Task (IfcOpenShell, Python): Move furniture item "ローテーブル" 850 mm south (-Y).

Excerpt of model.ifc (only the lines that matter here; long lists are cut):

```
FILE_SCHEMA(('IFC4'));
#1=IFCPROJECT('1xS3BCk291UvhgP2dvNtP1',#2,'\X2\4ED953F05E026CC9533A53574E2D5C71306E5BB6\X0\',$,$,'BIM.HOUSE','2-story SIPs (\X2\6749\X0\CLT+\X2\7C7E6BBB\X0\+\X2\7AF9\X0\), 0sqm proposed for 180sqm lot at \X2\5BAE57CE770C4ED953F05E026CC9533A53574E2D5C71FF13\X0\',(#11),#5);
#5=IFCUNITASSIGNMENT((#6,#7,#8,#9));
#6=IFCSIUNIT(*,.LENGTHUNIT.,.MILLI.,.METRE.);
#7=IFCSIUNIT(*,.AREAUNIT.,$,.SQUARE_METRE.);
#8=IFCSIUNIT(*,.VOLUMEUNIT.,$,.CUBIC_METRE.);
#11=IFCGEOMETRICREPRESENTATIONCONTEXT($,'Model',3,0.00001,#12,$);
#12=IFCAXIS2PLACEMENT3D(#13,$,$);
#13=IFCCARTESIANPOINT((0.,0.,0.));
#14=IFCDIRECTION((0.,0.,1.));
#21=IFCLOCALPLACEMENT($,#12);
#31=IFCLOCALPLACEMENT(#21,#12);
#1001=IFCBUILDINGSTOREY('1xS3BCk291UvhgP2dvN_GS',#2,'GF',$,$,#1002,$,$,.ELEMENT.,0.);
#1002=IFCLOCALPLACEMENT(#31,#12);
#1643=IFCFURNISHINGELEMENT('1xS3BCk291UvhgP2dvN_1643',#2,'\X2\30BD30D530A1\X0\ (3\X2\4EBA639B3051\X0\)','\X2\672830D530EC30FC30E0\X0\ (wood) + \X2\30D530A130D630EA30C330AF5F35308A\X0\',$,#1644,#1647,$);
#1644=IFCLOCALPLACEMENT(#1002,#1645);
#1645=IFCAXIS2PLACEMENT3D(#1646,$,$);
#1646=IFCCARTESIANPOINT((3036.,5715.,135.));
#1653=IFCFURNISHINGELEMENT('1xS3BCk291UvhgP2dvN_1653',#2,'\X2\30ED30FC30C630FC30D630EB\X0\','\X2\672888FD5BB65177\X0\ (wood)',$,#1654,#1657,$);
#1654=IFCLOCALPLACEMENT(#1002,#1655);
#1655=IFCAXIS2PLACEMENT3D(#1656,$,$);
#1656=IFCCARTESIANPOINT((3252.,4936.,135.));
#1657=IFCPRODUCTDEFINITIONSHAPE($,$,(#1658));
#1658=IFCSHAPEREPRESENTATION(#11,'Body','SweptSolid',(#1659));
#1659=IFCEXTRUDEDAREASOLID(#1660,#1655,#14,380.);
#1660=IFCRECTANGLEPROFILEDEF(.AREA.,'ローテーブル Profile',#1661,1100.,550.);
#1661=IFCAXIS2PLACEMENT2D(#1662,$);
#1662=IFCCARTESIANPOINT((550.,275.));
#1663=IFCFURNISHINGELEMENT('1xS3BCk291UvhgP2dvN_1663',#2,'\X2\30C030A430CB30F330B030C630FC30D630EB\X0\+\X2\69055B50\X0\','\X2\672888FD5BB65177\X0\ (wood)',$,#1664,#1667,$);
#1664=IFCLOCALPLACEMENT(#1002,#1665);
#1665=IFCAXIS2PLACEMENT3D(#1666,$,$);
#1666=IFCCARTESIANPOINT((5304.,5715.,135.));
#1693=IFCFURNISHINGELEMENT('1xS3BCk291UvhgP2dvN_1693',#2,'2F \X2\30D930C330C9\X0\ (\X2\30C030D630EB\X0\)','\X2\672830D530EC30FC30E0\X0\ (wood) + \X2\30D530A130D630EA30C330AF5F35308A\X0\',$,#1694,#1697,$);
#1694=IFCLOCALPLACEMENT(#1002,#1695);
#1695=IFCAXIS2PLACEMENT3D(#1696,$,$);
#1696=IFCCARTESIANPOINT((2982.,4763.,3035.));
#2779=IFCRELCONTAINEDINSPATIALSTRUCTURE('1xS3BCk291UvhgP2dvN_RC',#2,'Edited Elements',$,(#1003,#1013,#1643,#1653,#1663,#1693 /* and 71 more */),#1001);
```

```python
import ifcopenshell
import ifcopenshell.api.geometry
import ifcopenshell.util.placement
import ifcopenshell.util.unit

model = ifcopenshell.open("model.ifc")
unit_scale = ifcopenshell.util.unit.calculate_unit_scale(model)

item = model.by_guid("1xS3BCk291UvhgP2dvN_1653")
matrix = ifcopenshell.util.placement.get_local_placement(item.ObjectPlacement)
matrix[1, 3] -= 0.85 / unit_scale
ifcopenshell.api.geometry.edit_object_placement(model, product=item, matrix=matrix, is_si=False)

print(ifcopenshell.util.placement.get_local_placement(item.ObjectPlacement).round(3) + 0.0)

model.write("model_rev.ifc")
```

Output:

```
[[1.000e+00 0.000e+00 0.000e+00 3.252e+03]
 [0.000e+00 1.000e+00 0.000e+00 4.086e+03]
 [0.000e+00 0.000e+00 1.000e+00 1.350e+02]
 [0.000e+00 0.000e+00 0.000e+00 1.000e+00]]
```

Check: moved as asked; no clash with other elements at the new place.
